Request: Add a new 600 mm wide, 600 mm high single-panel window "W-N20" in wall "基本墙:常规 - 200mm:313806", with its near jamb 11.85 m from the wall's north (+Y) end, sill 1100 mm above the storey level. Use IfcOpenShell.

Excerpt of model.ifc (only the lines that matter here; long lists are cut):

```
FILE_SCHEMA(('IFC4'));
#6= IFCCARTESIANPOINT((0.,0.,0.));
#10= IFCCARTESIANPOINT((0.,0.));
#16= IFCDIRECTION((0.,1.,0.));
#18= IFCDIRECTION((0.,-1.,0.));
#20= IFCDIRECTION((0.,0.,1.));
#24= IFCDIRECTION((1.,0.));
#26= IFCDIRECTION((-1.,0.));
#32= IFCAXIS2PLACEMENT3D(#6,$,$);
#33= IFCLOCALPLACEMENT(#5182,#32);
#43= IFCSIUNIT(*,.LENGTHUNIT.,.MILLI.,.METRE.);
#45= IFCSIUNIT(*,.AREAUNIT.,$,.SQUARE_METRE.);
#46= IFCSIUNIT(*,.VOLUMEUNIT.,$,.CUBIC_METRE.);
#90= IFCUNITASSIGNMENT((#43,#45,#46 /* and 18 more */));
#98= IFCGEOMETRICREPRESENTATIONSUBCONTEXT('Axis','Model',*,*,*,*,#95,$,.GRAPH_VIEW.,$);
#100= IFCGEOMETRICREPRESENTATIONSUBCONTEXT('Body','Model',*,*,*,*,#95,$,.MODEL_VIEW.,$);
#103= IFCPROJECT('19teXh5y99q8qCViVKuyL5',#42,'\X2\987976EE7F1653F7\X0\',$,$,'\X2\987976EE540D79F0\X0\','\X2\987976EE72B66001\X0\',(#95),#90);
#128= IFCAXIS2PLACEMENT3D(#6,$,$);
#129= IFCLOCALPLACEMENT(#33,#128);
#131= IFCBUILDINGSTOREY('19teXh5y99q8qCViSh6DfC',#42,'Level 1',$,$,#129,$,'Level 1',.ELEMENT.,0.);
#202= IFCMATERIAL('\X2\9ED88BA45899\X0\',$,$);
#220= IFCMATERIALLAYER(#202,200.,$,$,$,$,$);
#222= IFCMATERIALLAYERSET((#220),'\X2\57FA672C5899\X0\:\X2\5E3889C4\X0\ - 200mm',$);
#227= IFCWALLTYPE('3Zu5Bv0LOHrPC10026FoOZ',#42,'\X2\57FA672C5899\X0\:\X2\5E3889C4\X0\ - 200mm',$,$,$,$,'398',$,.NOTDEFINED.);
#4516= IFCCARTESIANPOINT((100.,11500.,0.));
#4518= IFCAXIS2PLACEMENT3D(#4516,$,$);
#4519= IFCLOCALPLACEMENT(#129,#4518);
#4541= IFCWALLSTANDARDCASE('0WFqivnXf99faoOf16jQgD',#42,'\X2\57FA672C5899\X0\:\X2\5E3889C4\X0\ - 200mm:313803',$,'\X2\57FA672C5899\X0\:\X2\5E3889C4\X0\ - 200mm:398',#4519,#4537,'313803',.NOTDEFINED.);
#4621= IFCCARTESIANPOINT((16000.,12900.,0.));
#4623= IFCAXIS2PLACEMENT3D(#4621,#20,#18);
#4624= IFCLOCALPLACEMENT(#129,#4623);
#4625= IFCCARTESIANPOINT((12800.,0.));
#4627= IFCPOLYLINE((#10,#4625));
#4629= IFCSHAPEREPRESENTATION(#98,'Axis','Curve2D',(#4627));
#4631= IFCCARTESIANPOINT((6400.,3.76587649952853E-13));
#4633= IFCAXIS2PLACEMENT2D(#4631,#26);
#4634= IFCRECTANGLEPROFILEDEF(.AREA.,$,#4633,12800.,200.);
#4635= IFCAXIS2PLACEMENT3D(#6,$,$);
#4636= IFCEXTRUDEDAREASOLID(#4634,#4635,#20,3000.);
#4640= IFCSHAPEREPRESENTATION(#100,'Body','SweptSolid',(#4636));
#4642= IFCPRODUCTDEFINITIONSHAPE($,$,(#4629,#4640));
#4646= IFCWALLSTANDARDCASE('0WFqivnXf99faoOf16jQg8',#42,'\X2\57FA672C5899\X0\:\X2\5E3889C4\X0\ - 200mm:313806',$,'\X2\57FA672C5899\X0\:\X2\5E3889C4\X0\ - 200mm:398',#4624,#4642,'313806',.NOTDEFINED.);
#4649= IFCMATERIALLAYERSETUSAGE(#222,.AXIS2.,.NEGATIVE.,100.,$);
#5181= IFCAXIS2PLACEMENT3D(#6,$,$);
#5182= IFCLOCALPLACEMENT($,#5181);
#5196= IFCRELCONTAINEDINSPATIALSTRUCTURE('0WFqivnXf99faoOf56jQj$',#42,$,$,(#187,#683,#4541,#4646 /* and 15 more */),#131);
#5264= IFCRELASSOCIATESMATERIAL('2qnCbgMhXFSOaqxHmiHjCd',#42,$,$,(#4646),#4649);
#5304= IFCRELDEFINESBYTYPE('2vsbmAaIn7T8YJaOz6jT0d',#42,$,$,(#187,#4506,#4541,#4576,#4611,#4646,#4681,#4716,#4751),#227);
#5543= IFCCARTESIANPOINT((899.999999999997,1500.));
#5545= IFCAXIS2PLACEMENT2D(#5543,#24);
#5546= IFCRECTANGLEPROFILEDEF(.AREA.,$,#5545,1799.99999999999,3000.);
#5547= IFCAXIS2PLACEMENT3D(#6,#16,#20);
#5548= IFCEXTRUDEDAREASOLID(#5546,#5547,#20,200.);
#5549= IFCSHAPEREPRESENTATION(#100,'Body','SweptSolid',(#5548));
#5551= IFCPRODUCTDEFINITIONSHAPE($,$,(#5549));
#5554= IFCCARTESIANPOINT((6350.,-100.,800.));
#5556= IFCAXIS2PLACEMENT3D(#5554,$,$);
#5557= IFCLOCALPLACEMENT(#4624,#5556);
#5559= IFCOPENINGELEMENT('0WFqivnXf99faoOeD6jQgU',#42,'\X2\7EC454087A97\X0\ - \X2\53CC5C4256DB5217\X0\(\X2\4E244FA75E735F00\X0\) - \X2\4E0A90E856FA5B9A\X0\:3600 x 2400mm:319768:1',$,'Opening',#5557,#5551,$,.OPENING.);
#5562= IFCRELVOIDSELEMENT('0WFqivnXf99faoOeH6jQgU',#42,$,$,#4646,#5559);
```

```python
import numpy as np
import ifcopenshell
import ifcopenshell.api.feature
import ifcopenshell.api.geometry
import ifcopenshell.api.root
import ifcopenshell.api.spatial
import ifcopenshell.geom
import ifcopenshell.util.element
import ifcopenshell.util.placement
import ifcopenshell.util.representation
import ifcopenshell.util.shape
import ifcopenshell.util.unit

model = ifcopenshell.open("model.ifc")
unit_scale = ifcopenshell.util.unit.calculate_unit_scale(model)
settings = ifcopenshell.geom.settings()


def volume(element):
    """Net volume in cubic metres, openings subtracted."""
    shape = ifcopenshell.geom.create_shape(settings, element)
    return ifcopenshell.util.shape.get_volume(shape.geometry)


wall = model.by_guid("0WFqivnXf99faoOf16jQg8")
storey = ifcopenshell.util.element.get_container(wall, ifc_class="IfcBuildingStorey")
context = ifcopenshell.util.representation.get_context(model, "Model", "Body", "MODEL_VIEW")
before = volume(wall)

width, height, from_end, sill = 0.6, 0.6, 11.85, 1.1  # metres

# The wall runs along its own X axis, and the end named is its -X end.
wall_shape = ifcopenshell.geom.create_shape(settings, wall)
x, y, z = ifcopenshell.util.shape.get_vertices(wall_shape.geometry).T
start = x.min() + from_end
face, thickness = float(y.min()), float(y.max() - y.min())
wall_matrix = ifcopenshell.util.placement.get_local_placement(wall.ObjectPlacement)
level = ifcopenshell.util.placement.get_local_placement(storey.ObjectPlacement)[2, 3]


def in_wall(x, y):
    """Placement at x, y metres in the wall's axes, at sill height."""
    matrix = wall_matrix.copy()
    matrix[:, 3] = wall_matrix @ np.array([x / unit_scale, y / unit_scale, 0.0, 1.0])
    matrix[2, 3] = level + sill / unit_scale
    return matrix


# Opening: a box that overshoots both wall faces by 50 mm.
opening = ifcopenshell.api.root.create_entity(model, ifc_class="IfcOpeningElement", predefined_type="OPENING")
box = ifcopenshell.api.geometry.add_wall_representation(
    model, context=context, length=width, height=height, thickness=thickness + 0.1
)
ifcopenshell.api.geometry.assign_representation(model, product=opening, representation=box)
ifcopenshell.api.geometry.edit_object_placement(model, product=opening, matrix=in_wall(start, face - 0.05), is_si=False)
ifcopenshell.api.feature.add_feature(model, feature=opening, element=wall)

window = ifcopenshell.api.root.create_entity(model, ifc_class="IfcWindow", name="W-N20", predefined_type="WINDOW")
window.OverallWidth, window.OverallHeight = width / unit_scale, height / unit_scale
window.PartitioningType = "SINGLE_PANEL"
body = ifcopenshell.api.geometry.add_window_representation(
    model,
    context=context,
    overall_width=window.OverallWidth,
    overall_height=window.OverallHeight,
    partition_type="SINGLE_PANEL",
)
ifcopenshell.api.geometry.assign_representation(model, product=window, representation=body)
ifcopenshell.api.spatial.assign_container(model, products=[window], relating_structure=storey)
ifcopenshell.api.feature.add_filling(model, opening=opening, element=window)

# Centre the window in the wall's thickness.
ifcopenshell.api.geometry.edit_object_placement(model, product=window, matrix=in_wall(start, face), is_si=False)
window_shape = ifcopenshell.geom.create_shape(settings, window)
depth = ifcopenshell.util.shape.get_vertices(window_shape.geometry)[:, 1]
offset = face + thickness / 2 - (depth.min() + depth.max()) / 2
ifcopenshell.api.geometry.edit_object_placement(model, product=window, matrix=in_wall(start, offset), is_si=False)

after = volume(wall)

print(f"wall volume {before:.3f} -> {after:.3f} m3")

model.write("model-out.ifc")
```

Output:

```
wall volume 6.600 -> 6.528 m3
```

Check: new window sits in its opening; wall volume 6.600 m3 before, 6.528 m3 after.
